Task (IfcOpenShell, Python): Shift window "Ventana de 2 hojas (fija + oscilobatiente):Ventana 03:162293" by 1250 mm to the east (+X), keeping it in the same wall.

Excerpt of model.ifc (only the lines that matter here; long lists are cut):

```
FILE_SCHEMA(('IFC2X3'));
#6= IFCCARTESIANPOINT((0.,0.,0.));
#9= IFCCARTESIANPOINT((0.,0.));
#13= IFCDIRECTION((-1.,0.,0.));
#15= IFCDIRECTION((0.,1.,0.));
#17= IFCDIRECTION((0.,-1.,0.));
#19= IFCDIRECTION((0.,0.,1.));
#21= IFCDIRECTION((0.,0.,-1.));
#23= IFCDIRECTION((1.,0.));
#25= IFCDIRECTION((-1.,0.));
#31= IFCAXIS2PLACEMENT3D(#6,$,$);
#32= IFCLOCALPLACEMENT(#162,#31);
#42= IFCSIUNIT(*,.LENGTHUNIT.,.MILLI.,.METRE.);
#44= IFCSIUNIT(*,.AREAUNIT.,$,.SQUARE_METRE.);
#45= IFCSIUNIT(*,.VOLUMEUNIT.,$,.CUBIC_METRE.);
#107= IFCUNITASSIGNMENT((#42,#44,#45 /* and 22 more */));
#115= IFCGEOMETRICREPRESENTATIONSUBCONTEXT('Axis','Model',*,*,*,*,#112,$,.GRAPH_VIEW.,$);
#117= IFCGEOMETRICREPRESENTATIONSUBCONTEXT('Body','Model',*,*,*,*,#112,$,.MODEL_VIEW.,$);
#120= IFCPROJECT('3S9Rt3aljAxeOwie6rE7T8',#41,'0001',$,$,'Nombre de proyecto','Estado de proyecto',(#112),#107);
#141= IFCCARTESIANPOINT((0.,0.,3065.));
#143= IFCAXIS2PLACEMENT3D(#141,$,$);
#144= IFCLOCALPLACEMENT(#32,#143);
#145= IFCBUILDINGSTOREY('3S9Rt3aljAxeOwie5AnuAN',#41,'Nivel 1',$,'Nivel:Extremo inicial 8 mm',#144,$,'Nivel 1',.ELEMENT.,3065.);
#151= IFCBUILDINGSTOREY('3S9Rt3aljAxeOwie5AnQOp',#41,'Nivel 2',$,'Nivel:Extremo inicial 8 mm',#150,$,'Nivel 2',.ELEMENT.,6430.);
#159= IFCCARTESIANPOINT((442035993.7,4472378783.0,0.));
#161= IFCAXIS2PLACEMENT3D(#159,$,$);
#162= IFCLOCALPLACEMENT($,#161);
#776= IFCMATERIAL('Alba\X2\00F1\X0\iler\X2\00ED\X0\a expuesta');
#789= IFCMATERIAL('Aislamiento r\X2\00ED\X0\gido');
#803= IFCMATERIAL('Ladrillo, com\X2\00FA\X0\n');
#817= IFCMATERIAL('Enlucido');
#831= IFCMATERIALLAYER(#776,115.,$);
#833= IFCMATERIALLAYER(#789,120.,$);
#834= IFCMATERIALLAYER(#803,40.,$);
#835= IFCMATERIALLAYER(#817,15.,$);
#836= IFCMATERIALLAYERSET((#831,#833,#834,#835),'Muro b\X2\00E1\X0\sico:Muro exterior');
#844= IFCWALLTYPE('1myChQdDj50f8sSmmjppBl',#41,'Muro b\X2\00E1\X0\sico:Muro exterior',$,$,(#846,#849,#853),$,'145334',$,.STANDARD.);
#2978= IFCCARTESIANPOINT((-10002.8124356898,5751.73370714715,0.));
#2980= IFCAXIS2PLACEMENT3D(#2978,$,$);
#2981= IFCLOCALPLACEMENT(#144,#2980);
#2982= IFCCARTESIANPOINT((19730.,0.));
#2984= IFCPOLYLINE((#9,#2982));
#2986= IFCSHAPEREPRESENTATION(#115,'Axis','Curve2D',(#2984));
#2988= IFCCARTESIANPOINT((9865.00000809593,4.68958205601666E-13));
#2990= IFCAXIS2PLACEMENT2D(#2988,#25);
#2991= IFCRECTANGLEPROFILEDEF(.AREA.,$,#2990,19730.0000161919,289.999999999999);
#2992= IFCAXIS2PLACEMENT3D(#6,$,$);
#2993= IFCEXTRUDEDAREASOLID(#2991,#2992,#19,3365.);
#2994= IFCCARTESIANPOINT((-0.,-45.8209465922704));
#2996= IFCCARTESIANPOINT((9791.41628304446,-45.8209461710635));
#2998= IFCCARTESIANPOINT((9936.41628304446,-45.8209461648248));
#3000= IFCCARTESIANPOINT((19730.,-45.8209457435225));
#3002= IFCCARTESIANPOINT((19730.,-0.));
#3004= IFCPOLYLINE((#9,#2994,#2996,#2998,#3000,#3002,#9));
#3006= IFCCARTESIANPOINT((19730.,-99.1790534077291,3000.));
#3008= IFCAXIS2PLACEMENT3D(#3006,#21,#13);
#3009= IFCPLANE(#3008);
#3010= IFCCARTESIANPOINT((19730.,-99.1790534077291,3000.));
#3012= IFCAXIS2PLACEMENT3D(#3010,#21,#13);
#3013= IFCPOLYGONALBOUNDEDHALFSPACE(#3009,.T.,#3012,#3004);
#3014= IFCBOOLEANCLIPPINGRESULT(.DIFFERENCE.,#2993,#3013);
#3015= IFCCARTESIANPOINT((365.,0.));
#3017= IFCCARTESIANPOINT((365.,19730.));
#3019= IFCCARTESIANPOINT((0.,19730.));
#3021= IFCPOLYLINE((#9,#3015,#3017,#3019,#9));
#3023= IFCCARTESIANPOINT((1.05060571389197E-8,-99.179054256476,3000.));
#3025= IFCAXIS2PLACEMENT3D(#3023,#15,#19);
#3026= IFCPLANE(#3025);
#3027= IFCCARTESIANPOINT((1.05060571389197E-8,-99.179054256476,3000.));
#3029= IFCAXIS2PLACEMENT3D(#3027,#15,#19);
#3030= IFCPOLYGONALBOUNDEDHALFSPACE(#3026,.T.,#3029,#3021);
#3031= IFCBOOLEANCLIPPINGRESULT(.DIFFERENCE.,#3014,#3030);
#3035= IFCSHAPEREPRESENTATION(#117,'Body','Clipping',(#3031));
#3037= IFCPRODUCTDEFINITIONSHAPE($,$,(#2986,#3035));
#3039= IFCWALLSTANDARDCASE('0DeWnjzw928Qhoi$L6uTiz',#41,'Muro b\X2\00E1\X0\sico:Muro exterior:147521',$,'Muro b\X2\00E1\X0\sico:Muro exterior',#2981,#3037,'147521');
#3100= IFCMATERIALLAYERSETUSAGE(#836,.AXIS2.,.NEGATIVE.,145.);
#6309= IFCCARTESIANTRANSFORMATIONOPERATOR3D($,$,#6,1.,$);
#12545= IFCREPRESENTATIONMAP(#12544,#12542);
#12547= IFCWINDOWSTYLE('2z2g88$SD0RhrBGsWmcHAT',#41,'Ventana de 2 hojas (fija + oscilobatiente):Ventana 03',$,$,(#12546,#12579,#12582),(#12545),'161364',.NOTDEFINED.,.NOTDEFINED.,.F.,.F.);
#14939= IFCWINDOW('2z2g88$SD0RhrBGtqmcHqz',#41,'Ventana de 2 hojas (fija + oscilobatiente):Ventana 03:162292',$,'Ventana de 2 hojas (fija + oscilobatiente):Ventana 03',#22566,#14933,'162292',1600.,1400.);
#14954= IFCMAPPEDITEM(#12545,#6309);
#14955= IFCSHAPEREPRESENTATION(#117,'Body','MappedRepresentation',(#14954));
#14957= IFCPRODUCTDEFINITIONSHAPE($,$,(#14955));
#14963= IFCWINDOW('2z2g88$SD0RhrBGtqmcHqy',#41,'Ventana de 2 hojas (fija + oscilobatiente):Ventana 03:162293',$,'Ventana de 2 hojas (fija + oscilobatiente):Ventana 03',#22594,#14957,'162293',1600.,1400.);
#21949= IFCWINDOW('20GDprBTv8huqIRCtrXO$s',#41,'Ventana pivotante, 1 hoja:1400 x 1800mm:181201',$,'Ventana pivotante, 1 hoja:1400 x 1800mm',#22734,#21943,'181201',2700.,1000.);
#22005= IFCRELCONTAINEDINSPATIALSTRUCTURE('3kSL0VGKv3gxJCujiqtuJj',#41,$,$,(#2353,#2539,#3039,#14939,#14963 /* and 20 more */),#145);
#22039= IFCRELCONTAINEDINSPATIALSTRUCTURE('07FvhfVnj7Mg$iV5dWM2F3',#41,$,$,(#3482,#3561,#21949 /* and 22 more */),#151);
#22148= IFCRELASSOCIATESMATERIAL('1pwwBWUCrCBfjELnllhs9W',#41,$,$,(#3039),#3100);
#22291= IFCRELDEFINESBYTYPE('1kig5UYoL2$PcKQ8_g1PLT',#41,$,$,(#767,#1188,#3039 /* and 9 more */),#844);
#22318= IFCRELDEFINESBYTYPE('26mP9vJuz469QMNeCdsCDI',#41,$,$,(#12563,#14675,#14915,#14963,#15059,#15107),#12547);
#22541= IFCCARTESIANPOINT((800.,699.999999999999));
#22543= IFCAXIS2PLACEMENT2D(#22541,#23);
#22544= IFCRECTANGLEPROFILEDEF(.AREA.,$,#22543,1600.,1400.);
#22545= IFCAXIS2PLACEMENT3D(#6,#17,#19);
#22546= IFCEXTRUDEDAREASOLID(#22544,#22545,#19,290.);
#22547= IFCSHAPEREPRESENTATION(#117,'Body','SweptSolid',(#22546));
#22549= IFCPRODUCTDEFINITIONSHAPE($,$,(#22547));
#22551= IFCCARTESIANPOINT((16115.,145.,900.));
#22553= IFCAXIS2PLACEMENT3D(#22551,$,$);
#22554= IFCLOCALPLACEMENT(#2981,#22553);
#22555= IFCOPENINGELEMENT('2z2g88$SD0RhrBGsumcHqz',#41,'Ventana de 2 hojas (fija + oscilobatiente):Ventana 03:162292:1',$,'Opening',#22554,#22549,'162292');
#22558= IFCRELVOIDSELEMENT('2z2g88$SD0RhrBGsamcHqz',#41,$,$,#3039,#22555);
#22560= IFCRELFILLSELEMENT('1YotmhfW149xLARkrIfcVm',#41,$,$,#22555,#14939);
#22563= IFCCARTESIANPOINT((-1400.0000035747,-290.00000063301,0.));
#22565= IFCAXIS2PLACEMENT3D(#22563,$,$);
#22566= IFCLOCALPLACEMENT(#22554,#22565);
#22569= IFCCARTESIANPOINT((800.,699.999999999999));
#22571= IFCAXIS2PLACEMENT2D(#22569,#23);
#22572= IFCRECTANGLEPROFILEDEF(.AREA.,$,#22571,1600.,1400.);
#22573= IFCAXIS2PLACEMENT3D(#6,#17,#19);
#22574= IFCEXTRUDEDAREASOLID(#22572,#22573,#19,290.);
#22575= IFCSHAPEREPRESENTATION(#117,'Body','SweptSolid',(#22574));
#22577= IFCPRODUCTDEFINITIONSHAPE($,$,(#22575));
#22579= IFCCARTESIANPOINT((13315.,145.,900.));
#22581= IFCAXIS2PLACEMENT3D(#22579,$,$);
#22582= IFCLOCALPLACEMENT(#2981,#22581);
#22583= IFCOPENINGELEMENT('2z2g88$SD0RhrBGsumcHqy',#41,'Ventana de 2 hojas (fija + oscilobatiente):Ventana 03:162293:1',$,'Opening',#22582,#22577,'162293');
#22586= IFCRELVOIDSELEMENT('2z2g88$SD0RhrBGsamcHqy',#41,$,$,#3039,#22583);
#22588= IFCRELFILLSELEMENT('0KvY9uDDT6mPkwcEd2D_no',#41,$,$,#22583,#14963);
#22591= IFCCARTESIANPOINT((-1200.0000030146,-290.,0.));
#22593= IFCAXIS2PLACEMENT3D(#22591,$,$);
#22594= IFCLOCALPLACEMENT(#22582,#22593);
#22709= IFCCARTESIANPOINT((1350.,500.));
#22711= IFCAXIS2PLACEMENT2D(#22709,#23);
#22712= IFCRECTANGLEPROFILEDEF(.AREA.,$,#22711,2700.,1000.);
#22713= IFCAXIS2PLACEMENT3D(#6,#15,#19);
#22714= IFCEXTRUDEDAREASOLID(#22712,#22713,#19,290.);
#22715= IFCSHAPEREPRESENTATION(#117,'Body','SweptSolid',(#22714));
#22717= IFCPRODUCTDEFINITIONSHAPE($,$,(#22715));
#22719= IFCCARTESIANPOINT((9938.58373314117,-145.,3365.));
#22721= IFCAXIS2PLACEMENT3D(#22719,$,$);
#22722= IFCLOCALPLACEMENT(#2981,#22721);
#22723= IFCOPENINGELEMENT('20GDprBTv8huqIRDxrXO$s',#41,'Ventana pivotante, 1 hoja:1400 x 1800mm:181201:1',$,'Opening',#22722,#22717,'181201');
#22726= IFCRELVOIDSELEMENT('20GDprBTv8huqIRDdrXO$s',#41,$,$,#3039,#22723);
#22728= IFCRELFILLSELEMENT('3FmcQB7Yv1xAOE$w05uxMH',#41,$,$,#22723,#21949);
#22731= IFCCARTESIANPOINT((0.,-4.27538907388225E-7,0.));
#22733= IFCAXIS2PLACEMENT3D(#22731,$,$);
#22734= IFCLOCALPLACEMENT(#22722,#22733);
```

```python
import ifcopenshell
import ifcopenshell.api.geometry
import ifcopenshell.util.placement
import ifcopenshell.util.unit

model = ifcopenshell.open("model.ifc")
unit_scale = ifcopenshell.util.unit.calculate_unit_scale(model)

window = model.by_id(14963)
opening = window.FillsVoids[0].RelatingOpeningElement
wall = opening.VoidsElements[0].RelatingBuildingElement

wall_matrix = ifcopenshell.util.placement.get_local_placement(wall.ObjectPlacement)
shift = wall_matrix[:3, 0] * 1.25 / unit_scale
before = ifcopenshell.util.placement.get_local_placement(window.ObjectPlacement)[:3, 3].copy()

# The window is placed relative to its opening, so it follows when the opening moves.
matrix = ifcopenshell.util.placement.get_local_placement(opening.ObjectPlacement)
matrix[:3, 3] += shift
ifcopenshell.api.geometry.edit_object_placement(
    model, product=opening, matrix=matrix, is_si=False, should_transform_children=True
)

after = ifcopenshell.util.placement.get_local_placement(window.ObjectPlacement)[:3, 3]
print("window moved by", (after - before).round(3) + 0.0)

model.write("model_rev.ifc")
```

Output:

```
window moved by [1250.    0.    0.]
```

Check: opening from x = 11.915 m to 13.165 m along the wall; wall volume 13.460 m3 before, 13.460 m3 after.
